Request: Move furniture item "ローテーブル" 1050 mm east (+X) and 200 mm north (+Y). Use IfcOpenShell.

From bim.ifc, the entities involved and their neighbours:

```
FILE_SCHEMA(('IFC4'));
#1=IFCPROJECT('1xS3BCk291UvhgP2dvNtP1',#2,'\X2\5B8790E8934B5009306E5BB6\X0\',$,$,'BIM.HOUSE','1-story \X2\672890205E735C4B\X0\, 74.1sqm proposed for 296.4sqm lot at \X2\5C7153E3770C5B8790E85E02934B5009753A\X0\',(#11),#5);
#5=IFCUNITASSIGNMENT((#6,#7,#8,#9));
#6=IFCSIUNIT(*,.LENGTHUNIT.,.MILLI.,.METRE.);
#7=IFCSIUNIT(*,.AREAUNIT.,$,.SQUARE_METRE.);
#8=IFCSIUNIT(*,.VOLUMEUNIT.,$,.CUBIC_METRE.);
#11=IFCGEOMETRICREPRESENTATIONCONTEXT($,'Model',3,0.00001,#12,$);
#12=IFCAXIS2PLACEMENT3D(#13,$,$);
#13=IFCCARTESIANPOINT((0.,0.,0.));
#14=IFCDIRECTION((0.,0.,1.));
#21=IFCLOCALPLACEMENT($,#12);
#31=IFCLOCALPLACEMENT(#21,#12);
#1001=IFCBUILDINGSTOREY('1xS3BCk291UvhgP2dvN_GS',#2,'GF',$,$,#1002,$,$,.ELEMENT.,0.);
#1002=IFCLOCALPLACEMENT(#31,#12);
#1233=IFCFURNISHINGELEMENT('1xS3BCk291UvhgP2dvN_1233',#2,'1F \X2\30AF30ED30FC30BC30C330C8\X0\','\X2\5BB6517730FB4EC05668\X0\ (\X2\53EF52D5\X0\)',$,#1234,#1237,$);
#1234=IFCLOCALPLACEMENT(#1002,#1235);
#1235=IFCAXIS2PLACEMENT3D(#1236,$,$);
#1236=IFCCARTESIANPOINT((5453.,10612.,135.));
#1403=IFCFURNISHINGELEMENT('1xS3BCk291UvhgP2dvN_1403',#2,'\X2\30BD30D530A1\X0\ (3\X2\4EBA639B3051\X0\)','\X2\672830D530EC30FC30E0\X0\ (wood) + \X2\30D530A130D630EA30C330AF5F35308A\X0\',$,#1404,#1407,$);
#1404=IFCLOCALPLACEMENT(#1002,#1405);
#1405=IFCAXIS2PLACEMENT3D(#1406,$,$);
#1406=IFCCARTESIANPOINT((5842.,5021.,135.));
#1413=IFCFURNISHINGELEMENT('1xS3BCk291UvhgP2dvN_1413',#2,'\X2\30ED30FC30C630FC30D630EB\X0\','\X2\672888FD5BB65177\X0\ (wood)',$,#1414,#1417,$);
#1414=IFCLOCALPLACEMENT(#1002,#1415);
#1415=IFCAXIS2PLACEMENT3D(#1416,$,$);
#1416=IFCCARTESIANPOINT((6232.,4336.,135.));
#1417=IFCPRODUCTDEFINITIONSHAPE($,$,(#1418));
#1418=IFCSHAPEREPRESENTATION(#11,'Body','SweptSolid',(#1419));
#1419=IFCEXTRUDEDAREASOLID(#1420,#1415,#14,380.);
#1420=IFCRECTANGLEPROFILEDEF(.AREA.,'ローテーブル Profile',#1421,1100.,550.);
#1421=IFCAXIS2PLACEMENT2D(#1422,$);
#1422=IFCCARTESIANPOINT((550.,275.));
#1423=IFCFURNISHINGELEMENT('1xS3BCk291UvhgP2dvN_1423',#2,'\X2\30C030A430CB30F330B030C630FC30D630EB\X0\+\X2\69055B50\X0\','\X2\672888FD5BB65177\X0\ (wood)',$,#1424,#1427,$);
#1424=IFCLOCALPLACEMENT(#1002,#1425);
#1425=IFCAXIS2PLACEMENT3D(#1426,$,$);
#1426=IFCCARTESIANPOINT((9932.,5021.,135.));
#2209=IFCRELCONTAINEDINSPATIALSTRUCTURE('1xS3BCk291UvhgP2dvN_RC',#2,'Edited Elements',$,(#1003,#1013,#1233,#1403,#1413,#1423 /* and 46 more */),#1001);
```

```python
import ifcopenshell
import ifcopenshell.api.geometry
import ifcopenshell.util.placement
import ifcopenshell.util.unit

model = ifcopenshell.open("bim.ifc")
unit_scale = ifcopenshell.util.unit.calculate_unit_scale(model)

item = model.by_guid("1xS3BCk291UvhgP2dvN_1413")
matrix = ifcopenshell.util.placement.get_local_placement(item.ObjectPlacement)
matrix[0, 3] += 1.05 / unit_scale
matrix[1, 3] += 0.2 / unit_scale
ifcopenshell.api.geometry.edit_object_placement(model, product=item, matrix=matrix, is_si=False)

print(ifcopenshell.util.placement.get_local_placement(item.ObjectPlacement).round(3) + 0.0)

model.write("bim_edited.ifc")
```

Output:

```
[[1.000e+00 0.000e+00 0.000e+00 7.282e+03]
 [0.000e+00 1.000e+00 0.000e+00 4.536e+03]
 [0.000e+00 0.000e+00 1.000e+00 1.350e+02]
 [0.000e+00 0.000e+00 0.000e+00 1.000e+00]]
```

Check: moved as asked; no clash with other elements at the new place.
